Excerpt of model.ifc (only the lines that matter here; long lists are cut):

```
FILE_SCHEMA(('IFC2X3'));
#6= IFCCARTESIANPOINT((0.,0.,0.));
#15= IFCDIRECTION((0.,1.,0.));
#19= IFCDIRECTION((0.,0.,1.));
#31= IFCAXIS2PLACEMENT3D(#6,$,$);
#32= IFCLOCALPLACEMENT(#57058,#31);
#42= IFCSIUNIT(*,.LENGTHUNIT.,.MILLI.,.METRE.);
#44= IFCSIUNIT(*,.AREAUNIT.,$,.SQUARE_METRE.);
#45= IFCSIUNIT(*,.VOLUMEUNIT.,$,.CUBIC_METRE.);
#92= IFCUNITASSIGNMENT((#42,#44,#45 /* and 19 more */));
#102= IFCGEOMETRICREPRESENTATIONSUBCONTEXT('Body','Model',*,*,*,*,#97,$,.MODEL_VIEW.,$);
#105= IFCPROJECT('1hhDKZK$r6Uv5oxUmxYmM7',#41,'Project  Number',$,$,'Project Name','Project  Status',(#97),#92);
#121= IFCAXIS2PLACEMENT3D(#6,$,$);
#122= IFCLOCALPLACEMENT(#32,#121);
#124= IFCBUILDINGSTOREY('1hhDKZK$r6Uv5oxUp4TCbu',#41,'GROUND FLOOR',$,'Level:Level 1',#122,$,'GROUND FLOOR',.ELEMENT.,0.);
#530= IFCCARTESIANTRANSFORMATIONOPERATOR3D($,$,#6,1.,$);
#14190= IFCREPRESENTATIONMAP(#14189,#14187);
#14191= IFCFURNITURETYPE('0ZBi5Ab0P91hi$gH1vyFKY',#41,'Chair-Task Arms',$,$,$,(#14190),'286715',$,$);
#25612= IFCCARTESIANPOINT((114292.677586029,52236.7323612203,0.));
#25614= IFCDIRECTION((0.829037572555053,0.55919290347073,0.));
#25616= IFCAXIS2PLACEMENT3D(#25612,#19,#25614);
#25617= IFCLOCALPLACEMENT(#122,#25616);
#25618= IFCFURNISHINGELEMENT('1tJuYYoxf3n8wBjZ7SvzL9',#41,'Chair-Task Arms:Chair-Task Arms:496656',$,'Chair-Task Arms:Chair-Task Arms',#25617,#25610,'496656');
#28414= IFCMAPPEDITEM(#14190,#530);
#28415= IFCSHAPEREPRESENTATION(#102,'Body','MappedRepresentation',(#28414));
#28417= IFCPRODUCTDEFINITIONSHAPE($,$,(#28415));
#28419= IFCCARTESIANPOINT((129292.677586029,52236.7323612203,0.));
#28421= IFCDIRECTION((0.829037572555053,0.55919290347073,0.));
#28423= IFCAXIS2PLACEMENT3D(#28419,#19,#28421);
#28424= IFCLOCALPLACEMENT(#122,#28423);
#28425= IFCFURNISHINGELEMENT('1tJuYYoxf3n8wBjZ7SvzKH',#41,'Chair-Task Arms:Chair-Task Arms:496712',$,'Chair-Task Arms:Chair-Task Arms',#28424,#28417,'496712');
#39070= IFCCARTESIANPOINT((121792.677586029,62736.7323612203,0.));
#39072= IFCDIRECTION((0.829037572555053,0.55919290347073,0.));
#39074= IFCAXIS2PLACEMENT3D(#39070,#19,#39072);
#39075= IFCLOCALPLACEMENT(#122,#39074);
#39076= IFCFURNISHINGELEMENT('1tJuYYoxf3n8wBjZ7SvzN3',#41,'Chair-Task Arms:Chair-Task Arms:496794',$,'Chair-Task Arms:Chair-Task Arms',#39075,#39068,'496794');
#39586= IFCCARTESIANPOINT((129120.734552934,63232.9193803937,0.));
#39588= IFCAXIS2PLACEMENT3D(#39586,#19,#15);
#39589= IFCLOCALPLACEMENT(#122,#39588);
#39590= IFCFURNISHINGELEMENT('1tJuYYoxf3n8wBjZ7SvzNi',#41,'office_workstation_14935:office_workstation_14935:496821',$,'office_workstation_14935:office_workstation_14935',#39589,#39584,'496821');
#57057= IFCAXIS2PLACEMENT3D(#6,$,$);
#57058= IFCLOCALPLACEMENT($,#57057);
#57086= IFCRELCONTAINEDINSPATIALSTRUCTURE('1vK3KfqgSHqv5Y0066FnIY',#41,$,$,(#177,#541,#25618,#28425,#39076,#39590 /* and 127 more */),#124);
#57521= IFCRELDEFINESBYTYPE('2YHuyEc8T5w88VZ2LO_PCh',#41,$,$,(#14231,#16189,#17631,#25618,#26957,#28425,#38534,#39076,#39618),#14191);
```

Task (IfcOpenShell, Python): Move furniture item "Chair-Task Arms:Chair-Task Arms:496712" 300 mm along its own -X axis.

```python
import ifcopenshell
import ifcopenshell.api.geometry
import ifcopenshell.util.placement
import ifcopenshell.util.unit

model = ifcopenshell.open("model.ifc")
unit_scale = ifcopenshell.util.unit.calculate_unit_scale(model)

item = model.by_guid("1tJuYYoxf3n8wBjZ7SvzKH")
matrix = ifcopenshell.util.placement.get_local_placement(item.ObjectPlacement)
matrix[:3, 3] -= matrix[:3, 0] * 0.3 / unit_scale
ifcopenshell.api.geometry.edit_object_placement(model, product=item, matrix=matrix, is_si=False)

print(ifcopenshell.util.placement.get_local_placement(item.ObjectPlacement).round(3) + 0.0)

model.write("model_edited.ifc")
```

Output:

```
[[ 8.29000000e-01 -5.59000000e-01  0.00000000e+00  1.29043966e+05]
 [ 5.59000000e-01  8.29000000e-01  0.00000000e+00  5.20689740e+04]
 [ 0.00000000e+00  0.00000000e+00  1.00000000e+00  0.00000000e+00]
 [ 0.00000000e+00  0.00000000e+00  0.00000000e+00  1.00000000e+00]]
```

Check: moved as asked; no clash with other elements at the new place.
